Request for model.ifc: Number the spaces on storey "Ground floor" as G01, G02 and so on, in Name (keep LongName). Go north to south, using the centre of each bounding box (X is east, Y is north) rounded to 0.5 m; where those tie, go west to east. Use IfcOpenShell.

First a look at what the model holds.

```python
import ifcopenshell
import ifcopenshell.util.element
import ifcopenshell.util.placement

model = ifcopenshell.open("model.ifc")
print(model.schema)
storey = next(s for s in model.by_type("IfcBuildingStorey") if s.Name == "Ground floor")
spaces = [e for e in ifcopenshell.util.element.get_decomposition(storey) if e.is_a("IfcSpace")]
for e in sorted(spaces, key=lambda e: e.id()):
    origin = ifcopenshell.util.placement.get_local_placement(e.ObjectPlacement)[:3, 3]
    print(e.id(), e.Name, e.LongName, origin.round(2) + 0.0, sep=" | ")
```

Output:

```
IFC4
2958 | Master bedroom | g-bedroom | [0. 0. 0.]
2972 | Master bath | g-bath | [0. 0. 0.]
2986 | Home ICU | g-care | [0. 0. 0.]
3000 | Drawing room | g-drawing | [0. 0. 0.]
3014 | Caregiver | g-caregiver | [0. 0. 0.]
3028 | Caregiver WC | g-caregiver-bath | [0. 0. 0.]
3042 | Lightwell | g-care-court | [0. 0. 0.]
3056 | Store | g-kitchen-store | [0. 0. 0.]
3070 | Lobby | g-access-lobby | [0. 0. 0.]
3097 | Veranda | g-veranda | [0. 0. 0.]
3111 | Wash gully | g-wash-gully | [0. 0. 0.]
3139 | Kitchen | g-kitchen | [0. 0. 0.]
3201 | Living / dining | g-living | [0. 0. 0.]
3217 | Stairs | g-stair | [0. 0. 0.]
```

```python
import ifcopenshell
import ifcopenshell.geom
import ifcopenshell.util.element
import ifcopenshell.util.shape

model = ifcopenshell.open("model.ifc")
settings = ifcopenshell.geom.settings()
settings.set("use-world-coords", True)


def centre(element):
    shape = ifcopenshell.geom.create_shape(settings, element)
    return ifcopenshell.util.shape.get_bbox_centroid(shape.geometry)


storey = next(s for s in model.by_type("IfcBuildingStorey") if s.Name == "Ground floor")
spaces = [e for e in ifcopenshell.util.element.get_decomposition(storey) if e.is_a("IfcSpace")]

# Insertion points can sit at a corner or the storey origin, so sort by the geometry (in metres).
centres = {e: centre(e) for e in spaces}
spaces.sort(key=lambda e: (-round(centres[e][1] / 0.5), centres[e][0]))

for i, e in enumerate(spaces, start=1):
    number = f"G{i:02d}"
    e.Name = number
    print(e.id(), number)

model.write("model_edited.ifc")
```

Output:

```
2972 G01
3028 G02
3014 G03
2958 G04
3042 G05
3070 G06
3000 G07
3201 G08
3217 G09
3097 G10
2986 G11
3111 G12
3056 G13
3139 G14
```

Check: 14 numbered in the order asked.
